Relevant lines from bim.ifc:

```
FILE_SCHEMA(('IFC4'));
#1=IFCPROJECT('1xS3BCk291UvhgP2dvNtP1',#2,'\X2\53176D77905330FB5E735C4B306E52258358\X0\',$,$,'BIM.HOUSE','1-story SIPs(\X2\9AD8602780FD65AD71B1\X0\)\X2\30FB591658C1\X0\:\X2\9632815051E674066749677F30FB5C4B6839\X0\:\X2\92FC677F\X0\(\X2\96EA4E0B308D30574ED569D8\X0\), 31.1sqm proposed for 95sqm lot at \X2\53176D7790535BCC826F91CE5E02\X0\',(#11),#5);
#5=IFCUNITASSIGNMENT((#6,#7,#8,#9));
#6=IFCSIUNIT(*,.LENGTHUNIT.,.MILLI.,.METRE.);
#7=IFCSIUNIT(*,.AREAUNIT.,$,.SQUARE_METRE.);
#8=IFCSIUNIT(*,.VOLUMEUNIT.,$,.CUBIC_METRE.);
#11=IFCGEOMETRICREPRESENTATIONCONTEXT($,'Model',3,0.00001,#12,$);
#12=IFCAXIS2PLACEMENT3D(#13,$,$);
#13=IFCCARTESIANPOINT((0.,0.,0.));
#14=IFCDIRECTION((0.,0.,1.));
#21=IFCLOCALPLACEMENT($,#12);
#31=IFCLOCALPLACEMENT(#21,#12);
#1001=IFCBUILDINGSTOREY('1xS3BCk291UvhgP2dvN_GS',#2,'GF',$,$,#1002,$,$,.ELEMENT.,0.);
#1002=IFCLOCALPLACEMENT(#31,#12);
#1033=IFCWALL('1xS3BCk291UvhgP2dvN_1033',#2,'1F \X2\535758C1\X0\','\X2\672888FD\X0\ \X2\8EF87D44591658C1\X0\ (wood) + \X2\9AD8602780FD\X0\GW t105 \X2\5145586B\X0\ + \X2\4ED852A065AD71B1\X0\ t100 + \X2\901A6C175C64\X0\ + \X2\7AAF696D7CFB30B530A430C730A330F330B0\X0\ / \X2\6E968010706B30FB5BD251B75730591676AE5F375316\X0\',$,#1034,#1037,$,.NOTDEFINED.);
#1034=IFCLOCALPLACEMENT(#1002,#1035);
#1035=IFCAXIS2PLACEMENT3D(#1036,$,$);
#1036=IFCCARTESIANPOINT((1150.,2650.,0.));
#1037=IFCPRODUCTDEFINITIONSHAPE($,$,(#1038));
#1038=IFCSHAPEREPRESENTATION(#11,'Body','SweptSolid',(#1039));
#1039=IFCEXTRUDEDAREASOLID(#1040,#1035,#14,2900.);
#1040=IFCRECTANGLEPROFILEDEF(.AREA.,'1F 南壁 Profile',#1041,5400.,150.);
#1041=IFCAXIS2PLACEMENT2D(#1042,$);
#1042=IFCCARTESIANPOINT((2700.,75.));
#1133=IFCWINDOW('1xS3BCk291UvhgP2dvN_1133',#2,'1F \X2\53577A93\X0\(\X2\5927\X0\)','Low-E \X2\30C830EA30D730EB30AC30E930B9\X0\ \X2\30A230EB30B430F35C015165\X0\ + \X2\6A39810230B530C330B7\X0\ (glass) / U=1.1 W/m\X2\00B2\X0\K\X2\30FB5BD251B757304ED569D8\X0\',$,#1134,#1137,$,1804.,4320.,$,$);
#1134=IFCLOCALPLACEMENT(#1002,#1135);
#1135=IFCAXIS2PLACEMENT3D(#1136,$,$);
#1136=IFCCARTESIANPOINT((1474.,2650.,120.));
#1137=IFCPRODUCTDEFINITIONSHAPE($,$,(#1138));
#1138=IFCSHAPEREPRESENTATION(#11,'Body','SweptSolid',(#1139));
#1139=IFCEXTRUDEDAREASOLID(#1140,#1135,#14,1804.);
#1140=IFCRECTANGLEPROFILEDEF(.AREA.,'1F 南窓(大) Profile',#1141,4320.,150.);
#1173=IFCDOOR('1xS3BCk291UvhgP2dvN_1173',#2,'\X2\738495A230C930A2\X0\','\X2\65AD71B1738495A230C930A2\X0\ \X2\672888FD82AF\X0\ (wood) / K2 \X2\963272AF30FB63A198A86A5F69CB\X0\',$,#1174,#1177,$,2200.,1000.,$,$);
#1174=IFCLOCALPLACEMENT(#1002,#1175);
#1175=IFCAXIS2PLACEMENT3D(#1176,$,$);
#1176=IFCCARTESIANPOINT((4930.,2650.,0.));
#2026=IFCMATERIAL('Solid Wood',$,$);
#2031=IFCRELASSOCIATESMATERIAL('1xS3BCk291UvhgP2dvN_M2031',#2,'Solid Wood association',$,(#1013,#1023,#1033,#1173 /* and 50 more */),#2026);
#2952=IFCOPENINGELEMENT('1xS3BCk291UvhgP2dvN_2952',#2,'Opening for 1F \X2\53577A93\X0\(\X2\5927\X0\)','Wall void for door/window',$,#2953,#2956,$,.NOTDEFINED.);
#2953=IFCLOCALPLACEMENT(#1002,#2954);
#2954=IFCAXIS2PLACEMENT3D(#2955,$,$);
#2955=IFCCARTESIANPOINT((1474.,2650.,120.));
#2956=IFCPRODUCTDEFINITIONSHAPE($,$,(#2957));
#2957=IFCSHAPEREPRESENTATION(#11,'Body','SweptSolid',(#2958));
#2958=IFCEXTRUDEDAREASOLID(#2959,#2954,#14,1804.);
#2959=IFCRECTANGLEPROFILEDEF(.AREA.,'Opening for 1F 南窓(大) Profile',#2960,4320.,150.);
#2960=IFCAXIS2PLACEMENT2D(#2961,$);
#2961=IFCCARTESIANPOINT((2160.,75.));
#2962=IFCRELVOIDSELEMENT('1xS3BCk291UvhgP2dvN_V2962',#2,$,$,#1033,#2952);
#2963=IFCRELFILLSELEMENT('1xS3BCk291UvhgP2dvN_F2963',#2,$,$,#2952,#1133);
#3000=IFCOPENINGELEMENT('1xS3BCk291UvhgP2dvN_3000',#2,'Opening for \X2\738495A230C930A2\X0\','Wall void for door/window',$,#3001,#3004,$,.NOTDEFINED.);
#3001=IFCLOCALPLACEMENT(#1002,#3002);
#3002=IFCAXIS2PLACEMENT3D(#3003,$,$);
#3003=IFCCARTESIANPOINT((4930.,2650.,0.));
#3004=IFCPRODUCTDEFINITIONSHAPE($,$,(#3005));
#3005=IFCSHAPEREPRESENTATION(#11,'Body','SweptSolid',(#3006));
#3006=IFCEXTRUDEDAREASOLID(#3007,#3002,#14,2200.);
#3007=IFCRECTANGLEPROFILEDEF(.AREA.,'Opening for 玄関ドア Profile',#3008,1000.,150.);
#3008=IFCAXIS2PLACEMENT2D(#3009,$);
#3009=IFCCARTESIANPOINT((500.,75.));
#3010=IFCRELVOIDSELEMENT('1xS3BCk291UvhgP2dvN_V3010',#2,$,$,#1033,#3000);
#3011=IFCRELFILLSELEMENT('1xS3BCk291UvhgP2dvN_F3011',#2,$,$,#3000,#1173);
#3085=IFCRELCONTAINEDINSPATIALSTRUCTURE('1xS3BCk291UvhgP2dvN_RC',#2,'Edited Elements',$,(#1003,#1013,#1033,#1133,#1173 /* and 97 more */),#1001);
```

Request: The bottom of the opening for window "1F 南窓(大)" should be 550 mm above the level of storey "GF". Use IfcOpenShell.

```python
import numpy as np
import ifcopenshell
import ifcopenshell.api.geometry
import ifcopenshell.geom
import ifcopenshell.util.element
import ifcopenshell.util.placement
import ifcopenshell.util.shape
import ifcopenshell.util.unit

model = ifcopenshell.open("bim.ifc")
unit_scale = ifcopenshell.util.unit.calculate_unit_scale(model)

window = model.by_guid("1xS3BCk291UvhgP2dvN_1133")
opening = window.FillsVoids[0].RelatingOpeningElement
storey = ifcopenshell.util.element.get_container(window, ifc_class="IfcBuildingStorey")
level = ifcopenshell.util.placement.get_local_placement(storey.ObjectPlacement)[2, 3]

# The opening's origin need not be at the sill, so measure its lowest point.
shape = ifcopenshell.geom.create_shape(ifcopenshell.geom.settings(), opening)
bottom = ifcopenshell.util.shape.get_shape_bottom_elevation(shape, shape.geometry) / unit_scale
dz = level + 0.55 / unit_scale - bottom

shift = np.array([0.0, 0.0, dz])
# The window is not placed relative to its opening, so move both.
for product in (opening, window):
    matrix = ifcopenshell.util.placement.get_local_placement(product.ObjectPlacement)
    matrix[:3, 3] += shift
    ifcopenshell.api.geometry.edit_object_placement(model, product=product, matrix=matrix, is_si=False)

print(f"moved by {dz * unit_scale:+.3f} m")

model.write("bim-out.ifc")
```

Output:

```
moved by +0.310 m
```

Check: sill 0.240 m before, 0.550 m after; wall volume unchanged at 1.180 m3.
